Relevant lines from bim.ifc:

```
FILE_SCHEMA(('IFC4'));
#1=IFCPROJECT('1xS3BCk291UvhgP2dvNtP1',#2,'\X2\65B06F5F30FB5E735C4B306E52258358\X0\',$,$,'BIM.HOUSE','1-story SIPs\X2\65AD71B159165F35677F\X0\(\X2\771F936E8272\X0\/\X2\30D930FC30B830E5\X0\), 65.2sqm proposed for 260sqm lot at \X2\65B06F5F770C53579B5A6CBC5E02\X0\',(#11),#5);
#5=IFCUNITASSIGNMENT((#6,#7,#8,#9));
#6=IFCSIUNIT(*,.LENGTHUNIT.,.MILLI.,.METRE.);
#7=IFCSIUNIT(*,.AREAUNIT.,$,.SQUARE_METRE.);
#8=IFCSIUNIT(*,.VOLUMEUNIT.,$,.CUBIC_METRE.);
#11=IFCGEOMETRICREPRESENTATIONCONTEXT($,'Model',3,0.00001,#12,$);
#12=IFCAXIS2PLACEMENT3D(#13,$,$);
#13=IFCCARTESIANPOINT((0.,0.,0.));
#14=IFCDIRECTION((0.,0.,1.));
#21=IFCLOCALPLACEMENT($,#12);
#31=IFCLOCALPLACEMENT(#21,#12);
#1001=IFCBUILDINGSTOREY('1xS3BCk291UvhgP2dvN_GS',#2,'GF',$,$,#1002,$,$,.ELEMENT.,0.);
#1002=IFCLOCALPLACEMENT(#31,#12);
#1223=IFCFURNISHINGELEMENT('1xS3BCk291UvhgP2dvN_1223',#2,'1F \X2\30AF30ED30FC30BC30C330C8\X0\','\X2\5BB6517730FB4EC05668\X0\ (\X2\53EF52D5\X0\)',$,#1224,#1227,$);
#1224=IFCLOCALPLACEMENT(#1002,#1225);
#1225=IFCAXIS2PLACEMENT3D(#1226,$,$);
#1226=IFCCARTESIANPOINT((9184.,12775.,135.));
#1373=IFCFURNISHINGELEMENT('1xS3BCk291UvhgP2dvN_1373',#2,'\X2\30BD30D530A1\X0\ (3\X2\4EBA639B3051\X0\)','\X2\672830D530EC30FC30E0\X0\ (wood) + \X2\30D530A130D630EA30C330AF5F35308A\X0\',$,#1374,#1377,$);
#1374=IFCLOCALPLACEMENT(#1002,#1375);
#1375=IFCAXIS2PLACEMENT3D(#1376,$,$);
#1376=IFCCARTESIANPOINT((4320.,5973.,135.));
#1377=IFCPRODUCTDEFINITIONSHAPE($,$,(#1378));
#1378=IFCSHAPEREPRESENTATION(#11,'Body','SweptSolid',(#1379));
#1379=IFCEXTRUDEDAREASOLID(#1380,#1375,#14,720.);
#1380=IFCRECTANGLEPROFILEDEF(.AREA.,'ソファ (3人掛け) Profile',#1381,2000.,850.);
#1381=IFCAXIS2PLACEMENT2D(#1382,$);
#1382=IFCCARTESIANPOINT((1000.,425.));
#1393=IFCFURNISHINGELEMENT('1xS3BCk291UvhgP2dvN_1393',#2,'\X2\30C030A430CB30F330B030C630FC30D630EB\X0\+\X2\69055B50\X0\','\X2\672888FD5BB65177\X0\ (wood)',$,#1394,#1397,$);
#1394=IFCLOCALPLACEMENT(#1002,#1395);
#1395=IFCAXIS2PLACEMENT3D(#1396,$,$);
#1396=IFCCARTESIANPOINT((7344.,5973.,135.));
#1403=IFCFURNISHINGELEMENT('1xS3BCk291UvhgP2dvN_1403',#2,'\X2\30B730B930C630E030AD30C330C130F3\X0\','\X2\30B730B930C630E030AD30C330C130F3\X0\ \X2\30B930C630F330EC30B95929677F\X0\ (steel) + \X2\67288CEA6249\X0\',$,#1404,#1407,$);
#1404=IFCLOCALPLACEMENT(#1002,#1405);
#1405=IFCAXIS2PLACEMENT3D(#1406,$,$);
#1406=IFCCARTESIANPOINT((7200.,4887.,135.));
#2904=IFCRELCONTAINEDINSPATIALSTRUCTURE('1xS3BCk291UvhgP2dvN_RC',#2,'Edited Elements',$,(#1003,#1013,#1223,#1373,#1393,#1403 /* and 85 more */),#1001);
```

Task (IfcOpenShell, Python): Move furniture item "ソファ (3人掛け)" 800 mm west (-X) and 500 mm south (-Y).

```python
import ifcopenshell
import ifcopenshell.api.geometry
import ifcopenshell.util.placement
import ifcopenshell.util.unit

model = ifcopenshell.open("bim.ifc")
unit_scale = ifcopenshell.util.unit.calculate_unit_scale(model)

item = model.by_guid("1xS3BCk291UvhgP2dvN_1373")
matrix = ifcopenshell.util.placement.get_local_placement(item.ObjectPlacement)
matrix[0, 3] -= 0.8 / unit_scale
matrix[1, 3] -= 0.5 / unit_scale
ifcopenshell.api.geometry.edit_object_placement(model, product=item, matrix=matrix, is_si=False)

print(ifcopenshell.util.placement.get_local_placement(item.ObjectPlacement).round(3) + 0.0)

model.write("bim_v2.ifc")
```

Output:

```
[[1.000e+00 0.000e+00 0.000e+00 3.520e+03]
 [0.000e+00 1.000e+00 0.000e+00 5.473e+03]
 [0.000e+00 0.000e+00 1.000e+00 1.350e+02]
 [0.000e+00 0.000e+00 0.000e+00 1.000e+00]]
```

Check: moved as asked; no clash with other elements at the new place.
